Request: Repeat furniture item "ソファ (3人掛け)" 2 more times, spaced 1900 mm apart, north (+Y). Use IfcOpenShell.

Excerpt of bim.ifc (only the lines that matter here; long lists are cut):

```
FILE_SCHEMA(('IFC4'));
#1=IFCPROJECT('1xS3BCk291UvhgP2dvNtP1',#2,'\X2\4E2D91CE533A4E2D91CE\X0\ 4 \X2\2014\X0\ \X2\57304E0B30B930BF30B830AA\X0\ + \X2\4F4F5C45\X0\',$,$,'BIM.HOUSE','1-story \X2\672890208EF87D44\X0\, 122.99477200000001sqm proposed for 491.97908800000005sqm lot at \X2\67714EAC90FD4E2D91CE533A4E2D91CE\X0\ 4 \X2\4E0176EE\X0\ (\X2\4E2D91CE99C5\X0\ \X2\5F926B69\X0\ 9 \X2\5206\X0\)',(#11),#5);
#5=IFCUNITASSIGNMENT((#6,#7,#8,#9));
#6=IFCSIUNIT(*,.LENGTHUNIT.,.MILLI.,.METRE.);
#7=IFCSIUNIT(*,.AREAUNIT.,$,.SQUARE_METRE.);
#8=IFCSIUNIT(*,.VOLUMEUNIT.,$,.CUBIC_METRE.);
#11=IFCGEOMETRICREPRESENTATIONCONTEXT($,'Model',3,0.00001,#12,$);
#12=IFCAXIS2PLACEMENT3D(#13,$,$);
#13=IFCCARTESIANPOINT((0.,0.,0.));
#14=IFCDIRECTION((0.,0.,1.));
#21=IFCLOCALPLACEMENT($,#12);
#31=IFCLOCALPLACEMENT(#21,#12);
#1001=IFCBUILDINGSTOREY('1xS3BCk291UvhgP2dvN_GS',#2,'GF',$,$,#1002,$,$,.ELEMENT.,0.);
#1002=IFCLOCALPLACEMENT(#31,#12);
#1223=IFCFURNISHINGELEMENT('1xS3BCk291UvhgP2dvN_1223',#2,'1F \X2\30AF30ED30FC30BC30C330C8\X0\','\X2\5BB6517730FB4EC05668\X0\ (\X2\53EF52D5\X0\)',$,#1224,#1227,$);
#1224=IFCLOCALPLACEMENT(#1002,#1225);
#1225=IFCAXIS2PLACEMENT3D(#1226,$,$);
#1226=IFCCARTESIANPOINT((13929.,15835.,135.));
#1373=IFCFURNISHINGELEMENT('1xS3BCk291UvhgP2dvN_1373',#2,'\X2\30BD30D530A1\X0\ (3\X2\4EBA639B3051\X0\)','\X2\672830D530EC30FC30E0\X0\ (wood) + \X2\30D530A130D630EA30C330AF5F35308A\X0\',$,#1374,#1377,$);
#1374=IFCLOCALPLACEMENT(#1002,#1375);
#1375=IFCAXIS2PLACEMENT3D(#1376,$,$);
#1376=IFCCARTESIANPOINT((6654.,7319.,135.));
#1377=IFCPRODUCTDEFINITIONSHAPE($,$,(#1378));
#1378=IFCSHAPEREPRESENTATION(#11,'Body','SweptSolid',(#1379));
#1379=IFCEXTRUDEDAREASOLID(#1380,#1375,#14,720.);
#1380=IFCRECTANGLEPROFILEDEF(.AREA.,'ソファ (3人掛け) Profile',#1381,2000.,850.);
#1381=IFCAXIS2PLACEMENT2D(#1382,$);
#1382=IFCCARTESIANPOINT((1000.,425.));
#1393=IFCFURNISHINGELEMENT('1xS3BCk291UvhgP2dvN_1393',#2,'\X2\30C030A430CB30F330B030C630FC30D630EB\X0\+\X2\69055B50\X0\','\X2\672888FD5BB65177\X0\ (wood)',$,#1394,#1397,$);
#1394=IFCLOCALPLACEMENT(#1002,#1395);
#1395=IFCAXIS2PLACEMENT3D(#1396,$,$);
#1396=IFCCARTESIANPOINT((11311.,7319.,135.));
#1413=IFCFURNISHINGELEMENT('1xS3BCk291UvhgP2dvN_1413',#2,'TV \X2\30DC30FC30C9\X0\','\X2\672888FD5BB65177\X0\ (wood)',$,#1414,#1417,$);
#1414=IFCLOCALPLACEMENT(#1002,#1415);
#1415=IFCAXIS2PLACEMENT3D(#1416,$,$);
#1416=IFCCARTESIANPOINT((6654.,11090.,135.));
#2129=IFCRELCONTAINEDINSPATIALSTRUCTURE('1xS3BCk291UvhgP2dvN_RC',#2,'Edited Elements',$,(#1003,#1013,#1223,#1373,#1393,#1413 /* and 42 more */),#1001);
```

```python
import numpy as np
import ifcopenshell
import ifcopenshell.api.geometry
import ifcopenshell.api.root
import ifcopenshell.util.element
import ifcopenshell.util.placement
import ifcopenshell.util.unit

model = ifcopenshell.open("bim.ifc")
unit_scale = ifcopenshell.util.unit.calculate_unit_scale(model)


def reuse_history(source, copy):
    """copy_class also copies each property set's owner history, people and application; keep the originals."""
    for rel in copy.IsDefinedBy:
        if rel.is_a("IfcRelDefinesByProperties") and (history := rel.RelatingPropertyDefinition.OwnerHistory):
            rel.RelatingPropertyDefinition.OwnerHistory = source.OwnerHistory
            ifcopenshell.util.element.remove_deep2(model, history)


source = model.by_id(1373)
base = ifcopenshell.util.placement.get_local_placement(source.ObjectPlacement)
step = np.array([0.0, 1.0, 0.0]) * 1.9 / unit_scale

for i in range(1, 3):
    copy = ifcopenshell.api.root.copy_class(model, product=source)
    copy.Representation = ifcopenshell.util.element.copy_deep(
        model, source.Representation, exclude=["IfcGeometricRepresentationContext", "IfcRepresentationMap"]
    )
    reuse_history(source, copy)
    matrix = base.copy()
    matrix[:3, 3] += i * step
    print("added at", matrix[:3, 3].round(3) + 0.0)
    ifcopenshell.api.geometry.edit_object_placement(model, product=copy, matrix=matrix, is_si=False)

model.write("bim_rev.ifc")
```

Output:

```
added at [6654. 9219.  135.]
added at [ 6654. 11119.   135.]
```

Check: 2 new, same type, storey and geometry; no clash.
